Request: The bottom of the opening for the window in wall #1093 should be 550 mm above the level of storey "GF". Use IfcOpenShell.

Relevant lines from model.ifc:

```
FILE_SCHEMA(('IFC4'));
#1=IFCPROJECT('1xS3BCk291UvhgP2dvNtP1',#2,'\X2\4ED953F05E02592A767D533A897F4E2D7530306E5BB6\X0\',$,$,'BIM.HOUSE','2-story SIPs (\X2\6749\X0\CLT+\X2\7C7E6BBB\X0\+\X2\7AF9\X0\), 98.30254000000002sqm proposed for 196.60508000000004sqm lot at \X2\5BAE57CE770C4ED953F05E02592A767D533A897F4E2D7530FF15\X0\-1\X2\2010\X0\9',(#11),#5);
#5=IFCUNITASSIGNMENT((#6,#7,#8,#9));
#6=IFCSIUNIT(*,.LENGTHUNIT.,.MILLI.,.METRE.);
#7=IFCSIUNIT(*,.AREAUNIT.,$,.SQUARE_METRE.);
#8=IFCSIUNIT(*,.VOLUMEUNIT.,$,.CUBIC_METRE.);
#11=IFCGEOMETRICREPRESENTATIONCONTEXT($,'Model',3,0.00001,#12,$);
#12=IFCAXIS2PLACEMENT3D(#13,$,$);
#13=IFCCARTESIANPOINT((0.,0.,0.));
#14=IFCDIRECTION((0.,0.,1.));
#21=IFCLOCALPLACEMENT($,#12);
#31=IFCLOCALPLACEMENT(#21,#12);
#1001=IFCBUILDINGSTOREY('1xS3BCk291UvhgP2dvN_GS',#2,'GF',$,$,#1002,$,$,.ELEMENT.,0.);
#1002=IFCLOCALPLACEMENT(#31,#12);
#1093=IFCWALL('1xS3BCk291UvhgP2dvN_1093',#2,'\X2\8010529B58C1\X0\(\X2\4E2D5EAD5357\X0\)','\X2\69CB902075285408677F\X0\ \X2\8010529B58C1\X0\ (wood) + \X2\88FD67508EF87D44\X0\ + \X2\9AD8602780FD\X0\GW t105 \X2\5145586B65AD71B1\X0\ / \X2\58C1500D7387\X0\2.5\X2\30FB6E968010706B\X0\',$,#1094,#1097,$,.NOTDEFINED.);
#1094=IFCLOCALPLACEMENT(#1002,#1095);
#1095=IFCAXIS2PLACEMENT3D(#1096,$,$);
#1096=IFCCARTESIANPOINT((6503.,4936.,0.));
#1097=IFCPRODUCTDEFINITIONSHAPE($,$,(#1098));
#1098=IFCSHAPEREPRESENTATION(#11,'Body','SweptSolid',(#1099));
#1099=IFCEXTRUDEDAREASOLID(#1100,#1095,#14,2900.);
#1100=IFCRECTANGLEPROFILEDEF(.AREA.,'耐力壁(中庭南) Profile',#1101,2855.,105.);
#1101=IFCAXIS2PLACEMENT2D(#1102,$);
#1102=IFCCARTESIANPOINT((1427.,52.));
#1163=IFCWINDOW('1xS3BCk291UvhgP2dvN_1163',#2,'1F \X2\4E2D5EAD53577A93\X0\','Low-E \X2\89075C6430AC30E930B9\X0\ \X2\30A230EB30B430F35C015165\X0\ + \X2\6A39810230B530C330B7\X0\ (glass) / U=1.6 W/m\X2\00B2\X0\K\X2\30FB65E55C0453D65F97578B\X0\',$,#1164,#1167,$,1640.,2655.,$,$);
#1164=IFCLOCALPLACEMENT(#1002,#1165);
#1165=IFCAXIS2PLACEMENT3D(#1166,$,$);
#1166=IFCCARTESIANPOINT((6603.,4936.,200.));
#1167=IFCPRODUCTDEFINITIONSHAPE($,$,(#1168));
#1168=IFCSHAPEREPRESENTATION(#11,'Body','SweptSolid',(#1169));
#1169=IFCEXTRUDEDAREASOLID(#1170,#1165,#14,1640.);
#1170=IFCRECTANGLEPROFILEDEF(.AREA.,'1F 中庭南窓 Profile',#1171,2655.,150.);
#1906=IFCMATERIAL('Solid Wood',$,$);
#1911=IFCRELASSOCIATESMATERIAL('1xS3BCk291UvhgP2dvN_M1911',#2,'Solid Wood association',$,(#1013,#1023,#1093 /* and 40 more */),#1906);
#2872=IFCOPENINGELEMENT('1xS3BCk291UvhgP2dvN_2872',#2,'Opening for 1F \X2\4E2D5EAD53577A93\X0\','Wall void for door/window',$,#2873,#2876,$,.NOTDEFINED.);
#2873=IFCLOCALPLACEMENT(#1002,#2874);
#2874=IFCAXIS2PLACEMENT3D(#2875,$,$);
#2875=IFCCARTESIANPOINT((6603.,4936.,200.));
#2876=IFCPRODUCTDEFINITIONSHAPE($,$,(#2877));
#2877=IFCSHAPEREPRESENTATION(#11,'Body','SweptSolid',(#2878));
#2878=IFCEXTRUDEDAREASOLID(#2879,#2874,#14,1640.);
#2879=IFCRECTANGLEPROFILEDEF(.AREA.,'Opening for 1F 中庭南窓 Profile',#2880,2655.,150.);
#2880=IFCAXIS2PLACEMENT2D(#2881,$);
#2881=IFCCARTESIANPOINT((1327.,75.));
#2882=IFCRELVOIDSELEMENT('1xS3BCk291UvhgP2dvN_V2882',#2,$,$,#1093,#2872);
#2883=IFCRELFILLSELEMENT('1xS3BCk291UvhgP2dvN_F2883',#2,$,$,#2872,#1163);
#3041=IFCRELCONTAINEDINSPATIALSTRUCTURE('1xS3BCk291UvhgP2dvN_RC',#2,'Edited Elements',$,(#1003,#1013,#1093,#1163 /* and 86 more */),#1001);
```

```python
import numpy as np
import ifcopenshell
import ifcopenshell.api.geometry
import ifcopenshell.geom
import ifcopenshell.util.element
import ifcopenshell.util.placement
import ifcopenshell.util.shape
import ifcopenshell.util.unit

model = ifcopenshell.open("model.ifc")
unit_scale = ifcopenshell.util.unit.calculate_unit_scale(model)

window = model.by_guid("1xS3BCk291UvhgP2dvN_1163")
opening = window.FillsVoids[0].RelatingOpeningElement
storey = ifcopenshell.util.element.get_container(window, ifc_class="IfcBuildingStorey")
level = ifcopenshell.util.placement.get_local_placement(storey.ObjectPlacement)[2, 3]

# The opening's origin need not be at the sill, so measure its lowest point.
shape = ifcopenshell.geom.create_shape(ifcopenshell.geom.settings(), opening)
bottom = ifcopenshell.util.shape.get_shape_bottom_elevation(shape, shape.geometry) / unit_scale
dz = level + 0.55 / unit_scale - bottom

shift = np.array([0.0, 0.0, dz])
# The window is not placed relative to its opening, so move both.
for product in (opening, window):
    matrix = ifcopenshell.util.placement.get_local_placement(product.ObjectPlacement)
    matrix[:3, 3] += shift
    ifcopenshell.api.geometry.edit_object_placement(model, product=product, matrix=matrix, is_si=False)

print(f"moved by {dz * unit_scale:+.3f} m")

model.write("model_edited.ifc")
```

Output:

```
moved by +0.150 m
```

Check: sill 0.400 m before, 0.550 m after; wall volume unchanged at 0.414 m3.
